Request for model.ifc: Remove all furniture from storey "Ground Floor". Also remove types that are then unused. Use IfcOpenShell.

First a look at what the model holds.

```python
import ifcopenshell
import ifcopenshell.util.element

model = ifcopenshell.open("model.ifc")
print(model.schema)
storey = next(s for s in model.by_type("IfcBuildingStorey") if s.Name == "Ground Floor")
furniture = [e for e in ifcopenshell.util.element.get_decomposition(storey) if e.is_a("IfcFurnishingElement")]
seen = {}
for e in furniture:
    element_type = ifcopenshell.util.element.get_type(e)
    name = element_type.Name if element_type not in (None, e) else None
    seen[name] = seen.get(name, 0) + 1
for name, count in sorted(seen.items(), key=str):
    print(count, "x", name)
```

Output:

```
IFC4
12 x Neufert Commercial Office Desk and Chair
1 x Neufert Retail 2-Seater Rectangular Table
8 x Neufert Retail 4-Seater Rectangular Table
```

```python
import ifcopenshell
import ifcopenshell.api.root
import ifcopenshell.util.element

model = ifcopenshell.open("model.ifc")

storey = next(s for s in model.by_type("IfcBuildingStorey") if s.Name == "Ground Floor")
furniture = [e for e in ifcopenshell.util.element.get_decomposition(storey) if e.is_a("IfcFurnishingElement")]
types = {ifcopenshell.util.element.get_type(e) for e in furniture} - {None, *furniture}

for e in furniture:
    ifcopenshell.api.root.remove_product(model, product=e)
print(len(furniture), "removed")

unused = [t for t in types if not ifcopenshell.util.element.get_types(t)]
for t in unused:
    ifcopenshell.api.root.remove_product(model, product=t)
print(len(unused), "unused types removed")

model.write("model_updated.ifc")
```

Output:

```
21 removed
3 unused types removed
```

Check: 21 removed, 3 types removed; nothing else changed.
